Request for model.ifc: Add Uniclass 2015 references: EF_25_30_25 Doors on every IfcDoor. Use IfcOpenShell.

First a look at what the model holds.

```python
import ifcopenshell

model = ifcopenshell.open("model.ifc")
print(model.schema)
print("classifications:", [c.Name for c in model.by_type("IfcClassification")])
for ifc_class in ("IfcDoor", "IfcRoof", "IfcStair", "IfcWall", "IfcWindow"):
    print(ifc_class, len(model.by_type(ifc_class)))
```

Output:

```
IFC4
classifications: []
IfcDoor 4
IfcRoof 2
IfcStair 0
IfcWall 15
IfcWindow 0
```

```python
import ifcopenshell
import ifcopenshell.api.classification

model = ifcopenshell.open("model.ifc")

system = ifcopenshell.api.classification.add_classification(model, classification="Uniclass 2015")

codes = {
    "IfcDoor": ("EF_25_30_25", "Doors"),
}
for ifc_class, (code, name) in codes.items():
    products = model.by_type(ifc_class)
    ifcopenshell.api.classification.add_reference(
        model, products=products, classification=system, identification=code, name=name
    )
    print(code, len(products))

model.write("model_v2.ifc")
```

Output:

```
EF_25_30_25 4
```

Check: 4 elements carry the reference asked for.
